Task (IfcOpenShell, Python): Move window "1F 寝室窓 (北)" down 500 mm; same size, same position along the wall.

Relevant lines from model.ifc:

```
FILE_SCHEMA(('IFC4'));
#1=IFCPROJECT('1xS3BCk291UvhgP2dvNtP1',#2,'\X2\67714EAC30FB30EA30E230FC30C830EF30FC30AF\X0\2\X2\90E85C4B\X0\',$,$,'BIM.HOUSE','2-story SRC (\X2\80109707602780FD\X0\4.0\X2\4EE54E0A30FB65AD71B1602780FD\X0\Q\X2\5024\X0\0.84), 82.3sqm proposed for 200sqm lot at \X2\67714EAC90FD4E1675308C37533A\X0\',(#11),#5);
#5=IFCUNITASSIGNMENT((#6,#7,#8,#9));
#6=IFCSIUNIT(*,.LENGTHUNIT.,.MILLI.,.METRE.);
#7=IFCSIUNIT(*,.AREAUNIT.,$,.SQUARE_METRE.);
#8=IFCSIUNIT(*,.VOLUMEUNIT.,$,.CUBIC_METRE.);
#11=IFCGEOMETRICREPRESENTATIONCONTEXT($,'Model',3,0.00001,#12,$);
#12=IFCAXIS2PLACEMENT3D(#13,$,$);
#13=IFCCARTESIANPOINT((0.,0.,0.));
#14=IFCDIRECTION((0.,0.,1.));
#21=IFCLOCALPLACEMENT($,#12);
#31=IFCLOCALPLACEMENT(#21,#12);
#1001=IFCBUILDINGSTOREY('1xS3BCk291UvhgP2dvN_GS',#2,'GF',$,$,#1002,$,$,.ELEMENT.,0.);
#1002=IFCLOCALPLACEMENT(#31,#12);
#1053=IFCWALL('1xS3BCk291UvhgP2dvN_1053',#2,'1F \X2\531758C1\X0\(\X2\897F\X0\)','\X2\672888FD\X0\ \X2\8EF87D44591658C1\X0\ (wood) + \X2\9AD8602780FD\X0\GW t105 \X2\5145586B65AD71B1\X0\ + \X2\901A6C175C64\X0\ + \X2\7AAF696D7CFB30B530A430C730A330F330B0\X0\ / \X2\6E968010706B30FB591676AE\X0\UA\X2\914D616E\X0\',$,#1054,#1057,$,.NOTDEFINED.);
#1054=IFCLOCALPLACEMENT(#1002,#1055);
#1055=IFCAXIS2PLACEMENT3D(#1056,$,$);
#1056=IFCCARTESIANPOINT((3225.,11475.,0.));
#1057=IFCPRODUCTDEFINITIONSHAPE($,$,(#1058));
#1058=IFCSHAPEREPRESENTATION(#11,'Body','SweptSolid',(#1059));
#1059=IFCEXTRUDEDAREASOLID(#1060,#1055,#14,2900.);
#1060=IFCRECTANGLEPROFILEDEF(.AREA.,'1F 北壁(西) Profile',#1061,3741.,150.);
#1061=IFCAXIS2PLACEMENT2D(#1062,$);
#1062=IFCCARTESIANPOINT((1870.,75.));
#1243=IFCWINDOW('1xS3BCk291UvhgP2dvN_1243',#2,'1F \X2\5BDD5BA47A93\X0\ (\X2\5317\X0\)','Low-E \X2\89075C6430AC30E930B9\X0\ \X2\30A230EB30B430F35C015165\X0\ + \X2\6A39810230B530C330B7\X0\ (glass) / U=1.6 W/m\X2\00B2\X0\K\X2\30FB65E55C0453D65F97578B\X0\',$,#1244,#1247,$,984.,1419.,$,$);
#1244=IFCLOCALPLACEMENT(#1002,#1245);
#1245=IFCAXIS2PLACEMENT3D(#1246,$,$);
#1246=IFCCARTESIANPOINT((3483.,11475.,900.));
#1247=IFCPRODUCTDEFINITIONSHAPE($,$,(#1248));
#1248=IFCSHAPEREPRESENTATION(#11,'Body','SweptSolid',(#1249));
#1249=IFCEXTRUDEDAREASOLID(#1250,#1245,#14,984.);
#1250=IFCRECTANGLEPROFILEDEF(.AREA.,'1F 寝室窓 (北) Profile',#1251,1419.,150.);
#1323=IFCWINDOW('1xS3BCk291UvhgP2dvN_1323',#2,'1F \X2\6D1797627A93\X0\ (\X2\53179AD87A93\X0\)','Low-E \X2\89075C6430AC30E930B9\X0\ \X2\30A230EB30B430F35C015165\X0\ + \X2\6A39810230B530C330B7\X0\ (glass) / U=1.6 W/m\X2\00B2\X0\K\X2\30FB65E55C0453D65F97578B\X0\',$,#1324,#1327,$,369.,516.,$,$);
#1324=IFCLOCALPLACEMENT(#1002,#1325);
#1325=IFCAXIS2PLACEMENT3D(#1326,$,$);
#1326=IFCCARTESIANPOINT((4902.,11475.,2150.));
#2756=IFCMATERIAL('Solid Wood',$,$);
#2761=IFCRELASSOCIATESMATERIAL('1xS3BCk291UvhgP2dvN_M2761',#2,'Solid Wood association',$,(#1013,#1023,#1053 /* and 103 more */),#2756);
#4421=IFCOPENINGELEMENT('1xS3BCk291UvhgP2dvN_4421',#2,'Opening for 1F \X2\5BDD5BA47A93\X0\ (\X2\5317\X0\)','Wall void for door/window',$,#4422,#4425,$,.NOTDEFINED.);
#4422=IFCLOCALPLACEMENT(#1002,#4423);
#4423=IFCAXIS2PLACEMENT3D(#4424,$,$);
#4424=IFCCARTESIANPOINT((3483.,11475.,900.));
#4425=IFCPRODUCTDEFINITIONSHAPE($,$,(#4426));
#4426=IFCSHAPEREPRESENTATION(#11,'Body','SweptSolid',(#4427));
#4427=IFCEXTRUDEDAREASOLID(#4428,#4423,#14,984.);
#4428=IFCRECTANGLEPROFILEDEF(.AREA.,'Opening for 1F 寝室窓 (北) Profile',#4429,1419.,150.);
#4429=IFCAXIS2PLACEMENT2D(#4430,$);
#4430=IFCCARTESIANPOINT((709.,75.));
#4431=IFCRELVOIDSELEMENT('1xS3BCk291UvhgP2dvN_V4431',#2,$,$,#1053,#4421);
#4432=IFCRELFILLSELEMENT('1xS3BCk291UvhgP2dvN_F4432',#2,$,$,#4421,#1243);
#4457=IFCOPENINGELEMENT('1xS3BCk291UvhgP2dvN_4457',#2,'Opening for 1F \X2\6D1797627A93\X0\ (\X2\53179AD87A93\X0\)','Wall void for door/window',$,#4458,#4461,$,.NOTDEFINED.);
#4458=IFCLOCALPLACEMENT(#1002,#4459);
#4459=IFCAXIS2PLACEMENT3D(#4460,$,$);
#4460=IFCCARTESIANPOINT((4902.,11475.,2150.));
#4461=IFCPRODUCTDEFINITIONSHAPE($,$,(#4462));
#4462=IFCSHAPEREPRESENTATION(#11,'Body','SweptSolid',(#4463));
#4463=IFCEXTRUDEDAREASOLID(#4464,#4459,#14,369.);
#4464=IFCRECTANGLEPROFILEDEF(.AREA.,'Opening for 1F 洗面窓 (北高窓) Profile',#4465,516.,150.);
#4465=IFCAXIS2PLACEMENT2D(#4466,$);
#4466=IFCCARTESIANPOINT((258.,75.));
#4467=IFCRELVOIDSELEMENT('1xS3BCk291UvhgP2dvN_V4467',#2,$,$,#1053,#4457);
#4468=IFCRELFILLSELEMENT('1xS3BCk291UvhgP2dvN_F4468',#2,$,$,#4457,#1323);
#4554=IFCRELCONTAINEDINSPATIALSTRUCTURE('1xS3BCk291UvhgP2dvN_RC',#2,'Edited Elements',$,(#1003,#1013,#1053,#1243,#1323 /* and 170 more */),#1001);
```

```python
import numpy as np
import ifcopenshell
import ifcopenshell.api.geometry
import ifcopenshell.util.placement
import ifcopenshell.util.unit

model = ifcopenshell.open("model.ifc")
unit_scale = ifcopenshell.util.unit.calculate_unit_scale(model)

window = model.by_guid("1xS3BCk291UvhgP2dvN_1243")
opening = window.FillsVoids[0].RelatingOpeningElement
dz = -0.5 / unit_scale

shift = np.array([0.0, 0.0, dz])
# The window is not placed relative to its opening, so move both.
for product in (opening, window):
    matrix = ifcopenshell.util.placement.get_local_placement(product.ObjectPlacement)
    matrix[:3, 3] += shift
    ifcopenshell.api.geometry.edit_object_placement(model, product=product, matrix=matrix, is_si=False)

print(f"moved by {dz * unit_scale:+.3f} m")

model.write("model_updated.ifc")
```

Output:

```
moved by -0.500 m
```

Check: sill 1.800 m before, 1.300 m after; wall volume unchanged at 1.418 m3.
